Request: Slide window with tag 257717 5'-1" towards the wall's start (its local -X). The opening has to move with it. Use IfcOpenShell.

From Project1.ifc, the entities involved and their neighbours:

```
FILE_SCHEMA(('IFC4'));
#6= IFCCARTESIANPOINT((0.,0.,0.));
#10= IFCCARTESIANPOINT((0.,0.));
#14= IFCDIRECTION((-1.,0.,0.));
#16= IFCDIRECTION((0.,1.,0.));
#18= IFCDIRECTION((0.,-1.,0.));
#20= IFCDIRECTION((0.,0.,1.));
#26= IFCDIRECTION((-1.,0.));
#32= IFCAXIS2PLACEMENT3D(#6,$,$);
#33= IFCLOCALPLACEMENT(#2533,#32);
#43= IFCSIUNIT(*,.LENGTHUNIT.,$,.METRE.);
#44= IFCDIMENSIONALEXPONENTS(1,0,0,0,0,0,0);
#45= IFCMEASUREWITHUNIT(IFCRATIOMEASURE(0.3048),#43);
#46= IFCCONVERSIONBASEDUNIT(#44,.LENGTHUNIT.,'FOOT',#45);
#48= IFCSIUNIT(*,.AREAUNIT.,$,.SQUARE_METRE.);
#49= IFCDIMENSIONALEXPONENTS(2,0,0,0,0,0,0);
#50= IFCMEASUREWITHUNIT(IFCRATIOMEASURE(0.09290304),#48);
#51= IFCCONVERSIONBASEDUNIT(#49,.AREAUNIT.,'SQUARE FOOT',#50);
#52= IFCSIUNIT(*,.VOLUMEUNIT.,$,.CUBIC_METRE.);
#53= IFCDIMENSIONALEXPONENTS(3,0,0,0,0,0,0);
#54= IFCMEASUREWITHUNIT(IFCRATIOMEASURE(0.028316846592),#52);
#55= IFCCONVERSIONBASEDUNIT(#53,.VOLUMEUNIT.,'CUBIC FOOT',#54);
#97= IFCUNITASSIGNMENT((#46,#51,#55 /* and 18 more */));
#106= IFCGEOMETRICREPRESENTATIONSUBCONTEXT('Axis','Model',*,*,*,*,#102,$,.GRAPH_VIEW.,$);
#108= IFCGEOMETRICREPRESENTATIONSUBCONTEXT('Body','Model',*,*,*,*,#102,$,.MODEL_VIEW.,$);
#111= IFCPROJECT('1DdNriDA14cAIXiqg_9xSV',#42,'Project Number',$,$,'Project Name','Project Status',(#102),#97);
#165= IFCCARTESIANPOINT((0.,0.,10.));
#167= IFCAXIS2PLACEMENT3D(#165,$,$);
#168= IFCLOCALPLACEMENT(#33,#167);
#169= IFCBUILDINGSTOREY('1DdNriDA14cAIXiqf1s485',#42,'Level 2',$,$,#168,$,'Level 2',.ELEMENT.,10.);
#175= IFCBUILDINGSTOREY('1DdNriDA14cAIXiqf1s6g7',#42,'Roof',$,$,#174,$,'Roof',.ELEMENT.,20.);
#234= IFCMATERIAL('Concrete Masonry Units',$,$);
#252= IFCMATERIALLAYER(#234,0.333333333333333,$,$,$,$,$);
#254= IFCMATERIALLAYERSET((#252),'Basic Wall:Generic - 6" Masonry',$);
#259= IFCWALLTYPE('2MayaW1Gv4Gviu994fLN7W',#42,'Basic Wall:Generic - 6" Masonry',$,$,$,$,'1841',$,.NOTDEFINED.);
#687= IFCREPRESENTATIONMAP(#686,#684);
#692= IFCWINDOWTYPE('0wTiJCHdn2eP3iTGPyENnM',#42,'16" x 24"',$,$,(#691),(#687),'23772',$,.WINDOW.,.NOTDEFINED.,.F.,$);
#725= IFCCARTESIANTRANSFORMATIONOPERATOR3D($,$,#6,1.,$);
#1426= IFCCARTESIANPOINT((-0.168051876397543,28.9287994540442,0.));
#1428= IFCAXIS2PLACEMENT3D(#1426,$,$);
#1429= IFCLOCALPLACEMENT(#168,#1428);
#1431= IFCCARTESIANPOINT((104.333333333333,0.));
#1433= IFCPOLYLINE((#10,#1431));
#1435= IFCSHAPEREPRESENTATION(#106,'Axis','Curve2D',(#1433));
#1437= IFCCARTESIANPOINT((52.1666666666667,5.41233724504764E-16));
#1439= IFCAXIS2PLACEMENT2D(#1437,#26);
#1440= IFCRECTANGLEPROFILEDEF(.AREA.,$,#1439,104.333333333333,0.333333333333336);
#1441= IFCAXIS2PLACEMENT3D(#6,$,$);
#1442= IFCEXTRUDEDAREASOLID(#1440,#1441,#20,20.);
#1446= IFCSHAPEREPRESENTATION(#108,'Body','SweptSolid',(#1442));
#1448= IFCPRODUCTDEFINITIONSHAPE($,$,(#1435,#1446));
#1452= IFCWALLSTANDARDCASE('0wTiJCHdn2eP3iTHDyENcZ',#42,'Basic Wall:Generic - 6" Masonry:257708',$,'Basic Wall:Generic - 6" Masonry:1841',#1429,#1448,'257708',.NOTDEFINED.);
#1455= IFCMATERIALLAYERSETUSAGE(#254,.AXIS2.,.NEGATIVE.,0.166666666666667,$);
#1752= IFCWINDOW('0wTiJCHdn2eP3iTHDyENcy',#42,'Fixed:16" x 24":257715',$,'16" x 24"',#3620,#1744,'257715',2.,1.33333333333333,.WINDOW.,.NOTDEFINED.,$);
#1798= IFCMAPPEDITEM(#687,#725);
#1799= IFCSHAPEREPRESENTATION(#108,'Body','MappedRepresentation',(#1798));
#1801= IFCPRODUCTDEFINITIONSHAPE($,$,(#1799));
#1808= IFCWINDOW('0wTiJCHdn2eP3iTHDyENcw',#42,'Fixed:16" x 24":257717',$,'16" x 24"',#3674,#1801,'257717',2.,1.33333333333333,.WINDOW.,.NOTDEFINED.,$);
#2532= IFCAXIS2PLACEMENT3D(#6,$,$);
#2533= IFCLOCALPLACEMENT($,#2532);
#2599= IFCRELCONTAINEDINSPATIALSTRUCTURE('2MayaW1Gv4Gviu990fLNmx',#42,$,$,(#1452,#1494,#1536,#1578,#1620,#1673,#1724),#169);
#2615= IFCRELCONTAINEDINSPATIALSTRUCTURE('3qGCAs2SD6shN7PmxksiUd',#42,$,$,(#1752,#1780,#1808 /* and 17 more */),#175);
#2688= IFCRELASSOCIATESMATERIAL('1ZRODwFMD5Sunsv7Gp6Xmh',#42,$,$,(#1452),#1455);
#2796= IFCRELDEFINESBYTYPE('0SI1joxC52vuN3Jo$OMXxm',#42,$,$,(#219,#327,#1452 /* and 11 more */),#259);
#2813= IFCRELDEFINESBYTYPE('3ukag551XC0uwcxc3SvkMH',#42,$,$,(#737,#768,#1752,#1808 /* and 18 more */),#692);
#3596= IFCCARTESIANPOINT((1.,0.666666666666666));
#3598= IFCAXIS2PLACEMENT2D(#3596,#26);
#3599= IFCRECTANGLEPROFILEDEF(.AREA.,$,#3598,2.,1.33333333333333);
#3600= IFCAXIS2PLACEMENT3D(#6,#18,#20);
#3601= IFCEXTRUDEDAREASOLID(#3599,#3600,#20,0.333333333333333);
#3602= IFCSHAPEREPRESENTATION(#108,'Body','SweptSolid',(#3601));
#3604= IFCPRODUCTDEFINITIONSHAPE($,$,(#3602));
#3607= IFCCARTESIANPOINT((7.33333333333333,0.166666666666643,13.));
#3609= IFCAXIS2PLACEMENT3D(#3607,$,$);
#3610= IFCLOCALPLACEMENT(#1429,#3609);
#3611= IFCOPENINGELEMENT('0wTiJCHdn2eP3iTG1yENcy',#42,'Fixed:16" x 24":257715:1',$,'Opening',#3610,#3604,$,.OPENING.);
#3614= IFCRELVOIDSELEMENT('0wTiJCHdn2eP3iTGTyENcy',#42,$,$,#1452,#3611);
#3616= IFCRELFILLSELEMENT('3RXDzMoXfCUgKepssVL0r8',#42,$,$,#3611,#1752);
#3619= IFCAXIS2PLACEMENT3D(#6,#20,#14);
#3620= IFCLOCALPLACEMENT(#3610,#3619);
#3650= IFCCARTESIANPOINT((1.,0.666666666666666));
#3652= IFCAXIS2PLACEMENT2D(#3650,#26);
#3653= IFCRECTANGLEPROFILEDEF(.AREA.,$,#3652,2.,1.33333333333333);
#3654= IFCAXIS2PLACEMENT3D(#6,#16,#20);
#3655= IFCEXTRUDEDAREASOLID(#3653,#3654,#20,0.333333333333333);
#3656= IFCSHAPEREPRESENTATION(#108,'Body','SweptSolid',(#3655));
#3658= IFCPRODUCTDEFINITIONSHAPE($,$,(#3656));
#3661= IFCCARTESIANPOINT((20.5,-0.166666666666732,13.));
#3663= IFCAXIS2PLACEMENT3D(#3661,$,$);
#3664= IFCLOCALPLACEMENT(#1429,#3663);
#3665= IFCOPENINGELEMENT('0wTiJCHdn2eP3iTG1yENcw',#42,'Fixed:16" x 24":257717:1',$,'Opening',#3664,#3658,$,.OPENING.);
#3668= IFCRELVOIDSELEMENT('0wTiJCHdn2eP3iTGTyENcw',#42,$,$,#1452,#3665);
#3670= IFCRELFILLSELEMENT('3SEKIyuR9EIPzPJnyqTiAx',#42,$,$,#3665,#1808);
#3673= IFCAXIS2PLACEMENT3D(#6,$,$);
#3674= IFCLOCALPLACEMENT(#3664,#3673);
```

```python
import ifcopenshell
import ifcopenshell.api.geometry
import ifcopenshell.util.placement
import ifcopenshell.util.unit

model = ifcopenshell.open("Project1.ifc")
unit_scale = ifcopenshell.util.unit.calculate_unit_scale(model)

window = model.by_guid("0wTiJCHdn2eP3iTHDyENcw")
opening = window.FillsVoids[0].RelatingOpeningElement
wall = opening.VoidsElements[0].RelatingBuildingElement

wall_matrix = ifcopenshell.util.placement.get_local_placement(wall.ObjectPlacement)
shift = wall_matrix[:3, 0] * -61 * 0.0254 / unit_scale
before = ifcopenshell.util.placement.get_local_placement(window.ObjectPlacement)[:3, 3].copy()

# The window is placed relative to its opening, so it follows when the opening moves.
matrix = ifcopenshell.util.placement.get_local_placement(opening.ObjectPlacement)
matrix[:3, 3] += shift
ifcopenshell.api.geometry.edit_object_placement(
    model, product=opening, matrix=matrix, is_si=False, should_transform_children=True
)

after = ifcopenshell.util.placement.get_local_placement(window.ObjectPlacement)[:3, 3]
print("window moved by", (after - before).round(3) + 0.0)

model.write("Project1_updated.ifc")
```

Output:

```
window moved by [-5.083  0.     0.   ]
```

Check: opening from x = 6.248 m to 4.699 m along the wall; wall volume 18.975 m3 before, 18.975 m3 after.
